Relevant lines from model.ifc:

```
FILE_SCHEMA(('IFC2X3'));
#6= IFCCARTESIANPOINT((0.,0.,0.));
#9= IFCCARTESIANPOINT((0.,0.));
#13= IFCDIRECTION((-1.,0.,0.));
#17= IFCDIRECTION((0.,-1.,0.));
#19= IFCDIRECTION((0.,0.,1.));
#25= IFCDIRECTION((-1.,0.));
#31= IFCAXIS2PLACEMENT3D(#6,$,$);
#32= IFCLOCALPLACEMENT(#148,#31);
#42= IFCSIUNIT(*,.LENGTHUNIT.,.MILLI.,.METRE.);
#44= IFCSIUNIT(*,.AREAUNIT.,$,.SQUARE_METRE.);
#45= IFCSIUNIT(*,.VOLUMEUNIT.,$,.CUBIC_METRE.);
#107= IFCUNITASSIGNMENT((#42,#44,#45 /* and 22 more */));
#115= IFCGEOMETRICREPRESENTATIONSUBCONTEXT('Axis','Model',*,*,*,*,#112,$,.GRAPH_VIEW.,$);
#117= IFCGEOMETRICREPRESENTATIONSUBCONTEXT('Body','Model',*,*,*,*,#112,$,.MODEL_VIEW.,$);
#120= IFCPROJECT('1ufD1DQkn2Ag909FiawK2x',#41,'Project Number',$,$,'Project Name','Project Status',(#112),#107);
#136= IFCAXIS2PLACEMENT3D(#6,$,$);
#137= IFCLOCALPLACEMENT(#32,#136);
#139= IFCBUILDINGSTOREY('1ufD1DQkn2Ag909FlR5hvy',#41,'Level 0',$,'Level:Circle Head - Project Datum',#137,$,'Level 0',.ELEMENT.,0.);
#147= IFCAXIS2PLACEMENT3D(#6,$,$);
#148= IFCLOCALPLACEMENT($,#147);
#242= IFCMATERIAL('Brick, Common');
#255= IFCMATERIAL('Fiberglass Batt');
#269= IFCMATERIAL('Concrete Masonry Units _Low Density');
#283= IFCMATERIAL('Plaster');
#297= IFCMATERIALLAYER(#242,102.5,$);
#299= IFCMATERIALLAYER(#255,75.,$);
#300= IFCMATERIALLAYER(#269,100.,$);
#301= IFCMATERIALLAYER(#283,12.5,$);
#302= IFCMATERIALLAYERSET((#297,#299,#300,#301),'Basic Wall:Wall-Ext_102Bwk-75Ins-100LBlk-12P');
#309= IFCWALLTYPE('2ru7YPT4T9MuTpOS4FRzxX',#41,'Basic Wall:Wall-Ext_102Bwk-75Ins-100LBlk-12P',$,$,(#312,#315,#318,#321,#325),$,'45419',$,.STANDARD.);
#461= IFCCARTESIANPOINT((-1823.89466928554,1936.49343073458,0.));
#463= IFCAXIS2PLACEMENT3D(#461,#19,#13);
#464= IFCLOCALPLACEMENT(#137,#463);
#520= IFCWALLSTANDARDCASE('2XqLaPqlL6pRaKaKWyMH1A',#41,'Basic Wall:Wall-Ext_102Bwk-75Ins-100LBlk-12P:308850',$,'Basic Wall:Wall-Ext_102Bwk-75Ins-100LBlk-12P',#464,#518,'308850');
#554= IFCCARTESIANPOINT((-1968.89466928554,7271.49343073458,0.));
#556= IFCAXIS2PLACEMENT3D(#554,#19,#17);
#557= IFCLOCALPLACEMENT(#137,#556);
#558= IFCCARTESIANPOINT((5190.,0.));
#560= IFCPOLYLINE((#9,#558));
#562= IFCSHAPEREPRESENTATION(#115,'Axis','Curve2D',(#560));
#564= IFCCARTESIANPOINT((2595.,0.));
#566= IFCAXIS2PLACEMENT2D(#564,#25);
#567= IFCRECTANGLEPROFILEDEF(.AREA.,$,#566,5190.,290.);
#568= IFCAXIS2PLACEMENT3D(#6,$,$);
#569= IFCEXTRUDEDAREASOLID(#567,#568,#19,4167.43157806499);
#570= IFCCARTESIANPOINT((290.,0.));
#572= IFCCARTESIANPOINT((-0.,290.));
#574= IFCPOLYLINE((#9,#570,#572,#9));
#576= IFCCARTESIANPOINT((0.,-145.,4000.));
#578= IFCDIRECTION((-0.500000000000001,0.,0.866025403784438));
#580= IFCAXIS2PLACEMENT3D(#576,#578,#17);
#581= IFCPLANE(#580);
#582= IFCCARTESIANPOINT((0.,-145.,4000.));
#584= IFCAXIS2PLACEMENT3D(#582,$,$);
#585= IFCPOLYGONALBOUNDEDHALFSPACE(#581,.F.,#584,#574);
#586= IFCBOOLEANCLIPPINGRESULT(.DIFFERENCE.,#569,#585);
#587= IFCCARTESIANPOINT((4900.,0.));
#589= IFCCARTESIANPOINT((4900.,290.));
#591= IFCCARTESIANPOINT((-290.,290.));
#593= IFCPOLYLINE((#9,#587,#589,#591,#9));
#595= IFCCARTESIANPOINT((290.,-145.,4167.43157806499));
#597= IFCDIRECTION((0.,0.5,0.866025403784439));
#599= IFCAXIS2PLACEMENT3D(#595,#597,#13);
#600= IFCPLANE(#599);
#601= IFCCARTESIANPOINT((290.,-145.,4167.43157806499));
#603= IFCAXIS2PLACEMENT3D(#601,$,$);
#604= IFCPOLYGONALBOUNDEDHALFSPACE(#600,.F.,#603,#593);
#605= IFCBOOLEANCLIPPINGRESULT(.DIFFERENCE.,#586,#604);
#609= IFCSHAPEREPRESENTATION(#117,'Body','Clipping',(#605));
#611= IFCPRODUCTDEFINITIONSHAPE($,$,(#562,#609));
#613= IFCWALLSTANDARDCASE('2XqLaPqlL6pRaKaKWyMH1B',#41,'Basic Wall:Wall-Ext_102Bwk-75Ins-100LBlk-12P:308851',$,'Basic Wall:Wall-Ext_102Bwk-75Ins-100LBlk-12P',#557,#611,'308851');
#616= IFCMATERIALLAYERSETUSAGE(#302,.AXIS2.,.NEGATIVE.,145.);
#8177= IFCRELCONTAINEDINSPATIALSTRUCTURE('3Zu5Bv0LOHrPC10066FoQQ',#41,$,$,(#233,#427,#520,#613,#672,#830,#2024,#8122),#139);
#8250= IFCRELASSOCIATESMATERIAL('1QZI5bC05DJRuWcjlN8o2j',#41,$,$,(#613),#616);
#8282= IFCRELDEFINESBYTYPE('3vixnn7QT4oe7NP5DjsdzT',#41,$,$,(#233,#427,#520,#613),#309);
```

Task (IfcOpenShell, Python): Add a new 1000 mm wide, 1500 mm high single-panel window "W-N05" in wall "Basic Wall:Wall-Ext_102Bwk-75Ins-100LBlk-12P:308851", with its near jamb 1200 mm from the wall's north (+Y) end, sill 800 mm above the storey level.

```python
import numpy as np
import ifcopenshell
import ifcopenshell.api.feature
import ifcopenshell.api.geometry
import ifcopenshell.api.root
import ifcopenshell.api.spatial
import ifcopenshell.api.type
import ifcopenshell.geom
import ifcopenshell.util.element
import ifcopenshell.util.placement
import ifcopenshell.util.representation
import ifcopenshell.util.shape
import ifcopenshell.util.unit

model = ifcopenshell.open("model.ifc")
unit_scale = ifcopenshell.util.unit.calculate_unit_scale(model)
settings = ifcopenshell.geom.settings()


def volume(element):
    """Net volume in cubic metres, openings subtracted."""
    shape = ifcopenshell.geom.create_shape(settings, element)
    return ifcopenshell.util.shape.get_volume(shape.geometry)


wall = model.by_guid("2XqLaPqlL6pRaKaKWyMH1B")
storey = ifcopenshell.util.element.get_container(wall, ifc_class="IfcBuildingStorey")
context = ifcopenshell.util.representation.get_context(model, "Model", "Body", "MODEL_VIEW")
before = volume(wall)

width, height, from_end, sill = 1, 1.5, 1.2, 0.8  # metres

# The wall runs along its own X axis, and the end named is its -X end.
wall_shape = ifcopenshell.geom.create_shape(settings, wall)
x, y, z = ifcopenshell.util.shape.get_vertices(wall_shape.geometry).T
start = x.min() + from_end
face, thickness = float(y.min()), float(y.max() - y.min())
wall_matrix = ifcopenshell.util.placement.get_local_placement(wall.ObjectPlacement)
level = ifcopenshell.util.placement.get_local_placement(storey.ObjectPlacement)[2, 3]


def in_wall(x, y):
    """Placement at x, y metres in the wall's axes, at sill height."""
    matrix = wall_matrix.copy()
    matrix[:, 3] = wall_matrix @ np.array([x / unit_scale, y / unit_scale, 0.0, 1.0])
    matrix[2, 3] = level + sill / unit_scale
    return matrix


# Opening: a box that overshoots both wall faces by 50 mm.
opening = ifcopenshell.api.root.create_entity(model, ifc_class="IfcOpeningElement")
box = ifcopenshell.api.geometry.add_wall_representation(
    model, context=context, length=width, height=height, thickness=thickness + 0.1
)
ifcopenshell.api.geometry.assign_representation(model, product=opening, representation=box)
ifcopenshell.api.geometry.edit_object_placement(model, product=opening, matrix=in_wall(start, face - 0.05), is_si=False)
ifcopenshell.api.feature.add_feature(model, feature=opening, element=wall)

window = ifcopenshell.api.root.create_entity(model, ifc_class="IfcWindow", name="W-N05")
window.OverallWidth, window.OverallHeight = width / unit_scale, height / unit_scale
body = ifcopenshell.api.geometry.add_window_representation(
    model,
    context=context,
    overall_width=window.OverallWidth,
    overall_height=window.OverallHeight,
    partition_type="SINGLE_PANEL",
)
ifcopenshell.api.geometry.assign_representation(model, product=window, representation=body)
ifcopenshell.api.spatial.assign_container(model, products=[window], relating_structure=storey)
fills = ifcopenshell.api.feature.add_filling(model, opening=opening, element=window)
fills.OwnerHistory = window.OwnerHistory  # required in IFC2X3

# IFC2X3 keeps the operation on the window style.
style = ifcopenshell.api.root.create_entity(model, ifc_class="IfcWindowStyle", name="W-N05")
style.OperationType, style.ConstructionType = "SINGLE_PANEL", "NOTDEFINED"
style.ParameterTakesPrecedence = style.Sizeable = False
ifcopenshell.api.type.assign_type(model, related_objects=[window], relating_type=style)

# Centre the window in the wall's thickness.
ifcopenshell.api.geometry.edit_object_placement(model, product=window, matrix=in_wall(start, face), is_si=False)
window_shape = ifcopenshell.geom.create_shape(settings, window)
depth = ifcopenshell.util.shape.get_vertices(window_shape.geometry)[:, 1]
offset = face + thickness / 2 - (depth.min() + depth.max()) / 2
ifcopenshell.api.geometry.edit_object_placement(model, product=window, matrix=in_wall(start, offset), is_si=False)

after = volume(wall)

print(f"wall volume {before:.3f} -> {after:.3f} m3")

model.write("model-out.ifc")
```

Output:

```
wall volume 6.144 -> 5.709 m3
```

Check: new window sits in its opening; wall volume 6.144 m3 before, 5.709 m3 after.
